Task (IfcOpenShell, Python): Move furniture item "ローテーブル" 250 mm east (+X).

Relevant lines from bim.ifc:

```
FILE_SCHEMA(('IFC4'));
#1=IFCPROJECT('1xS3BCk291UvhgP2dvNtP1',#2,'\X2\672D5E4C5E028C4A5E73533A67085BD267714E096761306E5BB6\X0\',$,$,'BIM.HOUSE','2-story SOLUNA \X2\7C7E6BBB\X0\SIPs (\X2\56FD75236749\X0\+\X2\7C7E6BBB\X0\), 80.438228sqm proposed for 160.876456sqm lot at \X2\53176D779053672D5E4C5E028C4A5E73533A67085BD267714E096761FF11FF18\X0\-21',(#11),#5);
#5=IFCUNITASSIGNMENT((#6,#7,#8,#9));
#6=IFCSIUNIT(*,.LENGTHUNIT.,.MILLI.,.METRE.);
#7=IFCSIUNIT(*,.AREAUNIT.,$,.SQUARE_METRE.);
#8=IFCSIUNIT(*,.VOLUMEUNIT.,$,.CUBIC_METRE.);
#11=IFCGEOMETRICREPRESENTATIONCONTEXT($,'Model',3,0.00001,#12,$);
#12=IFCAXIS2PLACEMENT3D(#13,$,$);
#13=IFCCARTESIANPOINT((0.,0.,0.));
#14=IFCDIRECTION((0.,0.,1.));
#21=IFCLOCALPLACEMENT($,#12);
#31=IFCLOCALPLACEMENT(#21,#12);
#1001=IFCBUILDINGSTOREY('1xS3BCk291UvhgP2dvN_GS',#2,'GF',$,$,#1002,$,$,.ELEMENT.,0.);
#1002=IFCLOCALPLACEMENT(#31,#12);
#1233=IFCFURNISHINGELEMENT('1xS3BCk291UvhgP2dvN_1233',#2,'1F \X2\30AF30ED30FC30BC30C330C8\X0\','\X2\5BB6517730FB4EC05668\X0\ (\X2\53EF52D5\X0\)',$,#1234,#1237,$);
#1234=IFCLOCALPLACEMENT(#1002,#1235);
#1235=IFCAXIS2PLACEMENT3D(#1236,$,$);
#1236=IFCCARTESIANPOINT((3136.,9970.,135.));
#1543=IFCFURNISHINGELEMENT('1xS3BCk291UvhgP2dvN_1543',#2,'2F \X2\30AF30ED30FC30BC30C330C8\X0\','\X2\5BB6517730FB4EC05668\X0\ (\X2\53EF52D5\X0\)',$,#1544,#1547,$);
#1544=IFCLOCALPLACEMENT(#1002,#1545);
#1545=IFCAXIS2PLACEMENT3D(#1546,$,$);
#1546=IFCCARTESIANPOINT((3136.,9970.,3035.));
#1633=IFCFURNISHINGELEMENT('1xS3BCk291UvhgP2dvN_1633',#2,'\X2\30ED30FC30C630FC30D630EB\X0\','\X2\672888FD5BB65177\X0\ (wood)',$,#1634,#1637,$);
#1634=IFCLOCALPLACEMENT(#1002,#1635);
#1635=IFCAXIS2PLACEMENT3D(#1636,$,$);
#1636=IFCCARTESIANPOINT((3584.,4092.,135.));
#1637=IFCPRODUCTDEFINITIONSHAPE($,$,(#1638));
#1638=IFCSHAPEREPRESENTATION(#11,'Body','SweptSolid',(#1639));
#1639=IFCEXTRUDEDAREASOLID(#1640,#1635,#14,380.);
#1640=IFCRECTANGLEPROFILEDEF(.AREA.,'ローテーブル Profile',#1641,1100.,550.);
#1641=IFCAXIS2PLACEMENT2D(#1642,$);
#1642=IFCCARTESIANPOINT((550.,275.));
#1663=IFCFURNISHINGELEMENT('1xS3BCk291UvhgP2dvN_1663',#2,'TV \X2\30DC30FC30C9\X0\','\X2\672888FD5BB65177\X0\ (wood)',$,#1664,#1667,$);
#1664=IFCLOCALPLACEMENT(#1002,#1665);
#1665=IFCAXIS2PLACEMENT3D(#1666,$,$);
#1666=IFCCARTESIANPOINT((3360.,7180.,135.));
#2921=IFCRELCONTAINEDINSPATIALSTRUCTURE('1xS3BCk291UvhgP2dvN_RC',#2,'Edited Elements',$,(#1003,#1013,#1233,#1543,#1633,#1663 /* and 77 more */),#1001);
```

```python
import ifcopenshell
import ifcopenshell.api.geometry
import ifcopenshell.util.placement
import ifcopenshell.util.unit

model = ifcopenshell.open("bim.ifc")
unit_scale = ifcopenshell.util.unit.calculate_unit_scale(model)

item = model.by_id(1633)
matrix = ifcopenshell.util.placement.get_local_placement(item.ObjectPlacement)
matrix[0, 3] += 0.25 / unit_scale
ifcopenshell.api.geometry.edit_object_placement(model, product=item, matrix=matrix, is_si=False)

print(ifcopenshell.util.placement.get_local_placement(item.ObjectPlacement).round(3) + 0.0)

model.write("bim-out.ifc")
```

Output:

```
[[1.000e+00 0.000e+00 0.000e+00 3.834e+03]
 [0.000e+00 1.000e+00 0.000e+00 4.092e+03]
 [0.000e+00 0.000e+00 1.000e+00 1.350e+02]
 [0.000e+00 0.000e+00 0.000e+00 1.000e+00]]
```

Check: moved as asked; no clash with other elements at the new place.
